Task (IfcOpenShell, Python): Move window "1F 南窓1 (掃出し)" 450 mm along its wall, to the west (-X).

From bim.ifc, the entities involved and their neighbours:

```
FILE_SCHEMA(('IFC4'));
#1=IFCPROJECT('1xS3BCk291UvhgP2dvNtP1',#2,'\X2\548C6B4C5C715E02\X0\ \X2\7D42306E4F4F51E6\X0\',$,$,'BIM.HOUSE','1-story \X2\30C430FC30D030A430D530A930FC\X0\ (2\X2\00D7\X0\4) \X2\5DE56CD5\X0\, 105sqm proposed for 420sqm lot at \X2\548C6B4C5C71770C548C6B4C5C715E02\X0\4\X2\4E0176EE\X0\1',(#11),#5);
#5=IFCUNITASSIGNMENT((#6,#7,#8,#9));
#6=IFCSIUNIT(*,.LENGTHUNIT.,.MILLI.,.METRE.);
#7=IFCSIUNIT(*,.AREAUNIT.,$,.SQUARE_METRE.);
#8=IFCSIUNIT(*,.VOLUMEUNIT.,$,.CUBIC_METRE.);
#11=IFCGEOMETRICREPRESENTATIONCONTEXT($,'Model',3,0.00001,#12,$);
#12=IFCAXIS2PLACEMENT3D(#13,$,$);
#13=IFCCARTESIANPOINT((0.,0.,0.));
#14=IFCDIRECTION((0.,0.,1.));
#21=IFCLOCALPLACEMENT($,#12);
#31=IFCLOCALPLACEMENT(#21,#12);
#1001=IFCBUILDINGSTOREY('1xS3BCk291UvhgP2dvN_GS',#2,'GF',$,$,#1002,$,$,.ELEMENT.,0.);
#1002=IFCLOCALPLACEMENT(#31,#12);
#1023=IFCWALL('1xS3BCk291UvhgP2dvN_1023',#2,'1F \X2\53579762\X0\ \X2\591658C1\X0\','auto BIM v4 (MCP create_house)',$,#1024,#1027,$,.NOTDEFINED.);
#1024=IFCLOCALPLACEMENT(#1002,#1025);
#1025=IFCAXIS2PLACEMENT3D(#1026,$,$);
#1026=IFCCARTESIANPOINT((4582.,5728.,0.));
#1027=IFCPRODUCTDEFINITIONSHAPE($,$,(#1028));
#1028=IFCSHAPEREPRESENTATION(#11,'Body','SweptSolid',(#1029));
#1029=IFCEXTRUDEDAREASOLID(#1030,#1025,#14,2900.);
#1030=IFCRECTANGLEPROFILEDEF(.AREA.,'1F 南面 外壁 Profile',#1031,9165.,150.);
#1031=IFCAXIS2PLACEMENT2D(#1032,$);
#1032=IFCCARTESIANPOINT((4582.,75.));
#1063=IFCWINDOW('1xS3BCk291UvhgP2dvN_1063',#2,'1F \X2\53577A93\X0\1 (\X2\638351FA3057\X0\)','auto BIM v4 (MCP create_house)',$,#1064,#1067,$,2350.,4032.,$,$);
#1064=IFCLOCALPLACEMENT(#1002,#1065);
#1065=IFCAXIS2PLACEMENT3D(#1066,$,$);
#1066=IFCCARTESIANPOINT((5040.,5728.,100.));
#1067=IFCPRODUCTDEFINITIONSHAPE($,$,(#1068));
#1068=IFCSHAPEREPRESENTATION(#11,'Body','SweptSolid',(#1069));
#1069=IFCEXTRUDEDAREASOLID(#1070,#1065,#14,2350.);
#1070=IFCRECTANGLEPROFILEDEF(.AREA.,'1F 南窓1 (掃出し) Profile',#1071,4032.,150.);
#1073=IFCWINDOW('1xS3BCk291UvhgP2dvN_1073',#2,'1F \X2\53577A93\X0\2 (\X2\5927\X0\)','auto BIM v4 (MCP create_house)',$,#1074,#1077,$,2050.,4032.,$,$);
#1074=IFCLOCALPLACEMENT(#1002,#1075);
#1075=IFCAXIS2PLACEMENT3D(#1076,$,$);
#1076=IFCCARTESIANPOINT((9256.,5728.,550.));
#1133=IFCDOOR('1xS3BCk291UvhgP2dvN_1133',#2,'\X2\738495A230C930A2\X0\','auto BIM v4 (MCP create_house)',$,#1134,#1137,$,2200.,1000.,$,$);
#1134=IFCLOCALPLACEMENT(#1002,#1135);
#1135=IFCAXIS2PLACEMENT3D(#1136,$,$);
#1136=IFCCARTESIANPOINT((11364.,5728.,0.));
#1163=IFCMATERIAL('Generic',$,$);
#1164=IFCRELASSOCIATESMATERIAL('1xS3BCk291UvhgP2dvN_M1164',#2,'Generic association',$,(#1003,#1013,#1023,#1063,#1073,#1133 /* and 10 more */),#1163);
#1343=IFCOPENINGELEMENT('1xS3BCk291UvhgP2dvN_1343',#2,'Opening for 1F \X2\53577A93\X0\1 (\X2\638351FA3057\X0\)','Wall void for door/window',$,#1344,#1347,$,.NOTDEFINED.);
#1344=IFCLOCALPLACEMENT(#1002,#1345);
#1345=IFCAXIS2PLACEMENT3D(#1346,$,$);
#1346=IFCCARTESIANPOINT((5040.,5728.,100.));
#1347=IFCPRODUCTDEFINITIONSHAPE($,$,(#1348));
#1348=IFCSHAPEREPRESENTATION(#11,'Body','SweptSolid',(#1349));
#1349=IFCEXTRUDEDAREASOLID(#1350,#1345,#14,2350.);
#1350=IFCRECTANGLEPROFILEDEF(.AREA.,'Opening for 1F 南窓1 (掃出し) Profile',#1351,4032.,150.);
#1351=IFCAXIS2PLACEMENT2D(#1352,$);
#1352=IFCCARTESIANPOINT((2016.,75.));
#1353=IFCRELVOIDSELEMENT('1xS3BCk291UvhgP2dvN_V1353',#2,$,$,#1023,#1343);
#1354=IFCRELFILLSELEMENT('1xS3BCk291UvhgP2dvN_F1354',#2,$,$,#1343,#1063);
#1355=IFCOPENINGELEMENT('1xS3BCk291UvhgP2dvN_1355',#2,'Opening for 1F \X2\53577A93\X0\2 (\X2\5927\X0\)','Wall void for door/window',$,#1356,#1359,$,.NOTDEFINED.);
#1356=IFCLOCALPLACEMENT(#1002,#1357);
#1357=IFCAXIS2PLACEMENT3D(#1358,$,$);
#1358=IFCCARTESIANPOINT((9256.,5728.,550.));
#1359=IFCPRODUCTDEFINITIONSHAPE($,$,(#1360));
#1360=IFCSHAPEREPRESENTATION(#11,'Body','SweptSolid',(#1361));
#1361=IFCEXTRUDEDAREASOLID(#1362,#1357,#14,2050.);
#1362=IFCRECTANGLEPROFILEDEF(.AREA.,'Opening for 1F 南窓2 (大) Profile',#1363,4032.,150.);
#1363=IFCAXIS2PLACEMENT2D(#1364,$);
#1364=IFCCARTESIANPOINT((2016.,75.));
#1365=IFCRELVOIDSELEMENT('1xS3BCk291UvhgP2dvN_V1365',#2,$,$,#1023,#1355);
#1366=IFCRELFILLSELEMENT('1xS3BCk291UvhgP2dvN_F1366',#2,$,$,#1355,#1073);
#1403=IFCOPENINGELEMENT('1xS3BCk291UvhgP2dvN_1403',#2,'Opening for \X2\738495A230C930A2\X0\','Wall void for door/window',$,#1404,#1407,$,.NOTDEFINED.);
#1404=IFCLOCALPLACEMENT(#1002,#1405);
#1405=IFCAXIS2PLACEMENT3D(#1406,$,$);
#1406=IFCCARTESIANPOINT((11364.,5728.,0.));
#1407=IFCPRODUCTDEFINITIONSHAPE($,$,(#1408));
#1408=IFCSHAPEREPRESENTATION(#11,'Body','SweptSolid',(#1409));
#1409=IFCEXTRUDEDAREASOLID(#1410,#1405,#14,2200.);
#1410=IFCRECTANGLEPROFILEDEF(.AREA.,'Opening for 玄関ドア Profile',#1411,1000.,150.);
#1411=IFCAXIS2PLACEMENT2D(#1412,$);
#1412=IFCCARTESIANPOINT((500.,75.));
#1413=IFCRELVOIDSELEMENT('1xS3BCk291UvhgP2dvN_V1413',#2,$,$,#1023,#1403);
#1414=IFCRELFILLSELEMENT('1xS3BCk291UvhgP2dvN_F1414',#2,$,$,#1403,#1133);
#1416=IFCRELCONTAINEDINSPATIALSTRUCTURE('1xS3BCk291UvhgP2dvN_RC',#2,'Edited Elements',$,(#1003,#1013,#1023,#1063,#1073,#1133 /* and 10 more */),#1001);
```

```python
import ifcopenshell
import ifcopenshell.api.geometry
import ifcopenshell.util.placement

model = ifcopenshell.open("bim.ifc")

window = model.by_id(1063)
opening = window.FillsVoids[0].RelatingOpeningElement
wall = opening.VoidsElements[0].RelatingBuildingElement

wall_matrix = ifcopenshell.util.placement.get_local_placement(wall.ObjectPlacement)
shift = wall_matrix[:3, 0] * -450.0
before = ifcopenshell.util.placement.get_local_placement(window.ObjectPlacement)[:3, 3].copy()

# The window is not placed relative to its opening, so move both.
for product in (opening, window):
    matrix = ifcopenshell.util.placement.get_local_placement(product.ObjectPlacement)
    matrix[:3, 3] += shift
    ifcopenshell.api.geometry.edit_object_placement(model, product=product, matrix=matrix, is_si=False)

after = ifcopenshell.util.placement.get_local_placement(window.ObjectPlacement)[:3, 3]
print("window moved by", (after - before).round(3) + 0.0)

model.write("bim_v2.ifc")
```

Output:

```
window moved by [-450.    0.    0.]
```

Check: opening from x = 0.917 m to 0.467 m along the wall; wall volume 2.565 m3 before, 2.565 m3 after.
